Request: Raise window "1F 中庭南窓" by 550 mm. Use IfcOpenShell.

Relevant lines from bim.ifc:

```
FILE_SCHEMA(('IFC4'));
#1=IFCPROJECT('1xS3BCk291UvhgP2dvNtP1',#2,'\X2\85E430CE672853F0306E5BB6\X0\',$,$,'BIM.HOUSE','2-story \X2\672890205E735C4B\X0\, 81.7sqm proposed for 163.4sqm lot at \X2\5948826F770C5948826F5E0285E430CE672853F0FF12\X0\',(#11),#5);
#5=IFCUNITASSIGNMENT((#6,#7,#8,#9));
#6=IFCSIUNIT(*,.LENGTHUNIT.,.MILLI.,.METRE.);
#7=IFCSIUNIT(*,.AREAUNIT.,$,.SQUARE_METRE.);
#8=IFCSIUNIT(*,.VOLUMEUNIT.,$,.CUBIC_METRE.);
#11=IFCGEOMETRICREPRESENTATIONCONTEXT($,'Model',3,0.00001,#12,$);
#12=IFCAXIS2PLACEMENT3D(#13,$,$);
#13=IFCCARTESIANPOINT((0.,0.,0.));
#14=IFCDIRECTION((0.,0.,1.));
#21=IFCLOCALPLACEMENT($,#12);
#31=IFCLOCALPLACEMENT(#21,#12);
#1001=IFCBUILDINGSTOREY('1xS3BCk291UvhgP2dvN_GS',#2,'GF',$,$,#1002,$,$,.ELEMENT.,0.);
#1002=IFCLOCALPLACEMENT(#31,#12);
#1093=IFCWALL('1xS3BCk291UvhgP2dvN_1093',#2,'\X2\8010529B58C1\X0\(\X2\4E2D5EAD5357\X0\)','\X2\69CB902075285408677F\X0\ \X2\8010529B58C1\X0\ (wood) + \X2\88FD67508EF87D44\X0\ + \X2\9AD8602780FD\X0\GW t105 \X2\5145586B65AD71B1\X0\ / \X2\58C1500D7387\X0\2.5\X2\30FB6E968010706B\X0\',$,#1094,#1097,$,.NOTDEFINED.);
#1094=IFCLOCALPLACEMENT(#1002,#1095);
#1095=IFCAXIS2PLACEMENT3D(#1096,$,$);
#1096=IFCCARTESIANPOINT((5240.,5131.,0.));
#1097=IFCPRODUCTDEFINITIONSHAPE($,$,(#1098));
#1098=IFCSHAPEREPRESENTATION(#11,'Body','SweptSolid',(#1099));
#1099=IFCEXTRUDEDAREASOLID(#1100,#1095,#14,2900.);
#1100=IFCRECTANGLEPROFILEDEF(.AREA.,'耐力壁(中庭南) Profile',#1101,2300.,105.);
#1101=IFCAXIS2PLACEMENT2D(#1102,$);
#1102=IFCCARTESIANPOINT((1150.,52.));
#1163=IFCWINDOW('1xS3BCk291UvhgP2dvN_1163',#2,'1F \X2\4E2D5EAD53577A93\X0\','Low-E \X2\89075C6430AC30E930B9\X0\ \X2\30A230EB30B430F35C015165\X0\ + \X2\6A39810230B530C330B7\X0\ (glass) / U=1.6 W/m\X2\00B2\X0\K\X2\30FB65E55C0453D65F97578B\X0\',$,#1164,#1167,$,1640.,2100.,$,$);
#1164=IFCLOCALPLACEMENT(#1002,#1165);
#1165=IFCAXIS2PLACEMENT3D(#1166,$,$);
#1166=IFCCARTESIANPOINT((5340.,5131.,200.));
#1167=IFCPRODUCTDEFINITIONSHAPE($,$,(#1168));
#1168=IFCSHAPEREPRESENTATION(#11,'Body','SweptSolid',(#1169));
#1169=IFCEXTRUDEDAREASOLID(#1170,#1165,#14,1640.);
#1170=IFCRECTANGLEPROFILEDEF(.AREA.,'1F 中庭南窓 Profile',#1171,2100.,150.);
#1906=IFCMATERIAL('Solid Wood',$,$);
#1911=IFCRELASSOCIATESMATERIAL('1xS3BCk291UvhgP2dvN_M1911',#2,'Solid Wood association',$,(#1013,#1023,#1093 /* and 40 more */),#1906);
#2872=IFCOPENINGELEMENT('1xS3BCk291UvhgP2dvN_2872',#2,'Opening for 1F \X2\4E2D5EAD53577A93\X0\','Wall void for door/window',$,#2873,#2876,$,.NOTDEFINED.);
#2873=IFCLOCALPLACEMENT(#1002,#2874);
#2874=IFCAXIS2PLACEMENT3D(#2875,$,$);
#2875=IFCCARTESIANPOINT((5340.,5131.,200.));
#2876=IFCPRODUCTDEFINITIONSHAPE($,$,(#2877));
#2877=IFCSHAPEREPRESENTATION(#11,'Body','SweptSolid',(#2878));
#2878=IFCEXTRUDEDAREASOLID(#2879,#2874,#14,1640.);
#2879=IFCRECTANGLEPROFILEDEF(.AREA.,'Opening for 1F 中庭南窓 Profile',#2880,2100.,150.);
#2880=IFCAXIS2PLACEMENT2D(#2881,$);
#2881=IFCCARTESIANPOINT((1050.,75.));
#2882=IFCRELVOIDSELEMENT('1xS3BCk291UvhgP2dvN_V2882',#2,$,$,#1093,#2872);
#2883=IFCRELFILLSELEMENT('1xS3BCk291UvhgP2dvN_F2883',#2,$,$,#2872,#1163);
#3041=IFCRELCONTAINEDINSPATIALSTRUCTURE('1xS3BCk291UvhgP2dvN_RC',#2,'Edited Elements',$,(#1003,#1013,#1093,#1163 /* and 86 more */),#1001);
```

```python
import numpy as np
import ifcopenshell
import ifcopenshell.api.geometry
import ifcopenshell.util.placement
import ifcopenshell.util.unit

model = ifcopenshell.open("bim.ifc")
unit_scale = ifcopenshell.util.unit.calculate_unit_scale(model)

window = model.by_id(1163)
opening = window.FillsVoids[0].RelatingOpeningElement
dz = 550.0

shift = np.array([0.0, 0.0, dz])
# The window is not placed relative to its opening, so move both.
for product in (opening, window):
    matrix = ifcopenshell.util.placement.get_local_placement(product.ObjectPlacement)
    matrix[:3, 3] += shift
    ifcopenshell.api.geometry.edit_object_placement(model, product=product, matrix=matrix, is_si=False)

print(f"moved by {dz * unit_scale:+.3f} m")

model.write("bim_rev.ifc")
```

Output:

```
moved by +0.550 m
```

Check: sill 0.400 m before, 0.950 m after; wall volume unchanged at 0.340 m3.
